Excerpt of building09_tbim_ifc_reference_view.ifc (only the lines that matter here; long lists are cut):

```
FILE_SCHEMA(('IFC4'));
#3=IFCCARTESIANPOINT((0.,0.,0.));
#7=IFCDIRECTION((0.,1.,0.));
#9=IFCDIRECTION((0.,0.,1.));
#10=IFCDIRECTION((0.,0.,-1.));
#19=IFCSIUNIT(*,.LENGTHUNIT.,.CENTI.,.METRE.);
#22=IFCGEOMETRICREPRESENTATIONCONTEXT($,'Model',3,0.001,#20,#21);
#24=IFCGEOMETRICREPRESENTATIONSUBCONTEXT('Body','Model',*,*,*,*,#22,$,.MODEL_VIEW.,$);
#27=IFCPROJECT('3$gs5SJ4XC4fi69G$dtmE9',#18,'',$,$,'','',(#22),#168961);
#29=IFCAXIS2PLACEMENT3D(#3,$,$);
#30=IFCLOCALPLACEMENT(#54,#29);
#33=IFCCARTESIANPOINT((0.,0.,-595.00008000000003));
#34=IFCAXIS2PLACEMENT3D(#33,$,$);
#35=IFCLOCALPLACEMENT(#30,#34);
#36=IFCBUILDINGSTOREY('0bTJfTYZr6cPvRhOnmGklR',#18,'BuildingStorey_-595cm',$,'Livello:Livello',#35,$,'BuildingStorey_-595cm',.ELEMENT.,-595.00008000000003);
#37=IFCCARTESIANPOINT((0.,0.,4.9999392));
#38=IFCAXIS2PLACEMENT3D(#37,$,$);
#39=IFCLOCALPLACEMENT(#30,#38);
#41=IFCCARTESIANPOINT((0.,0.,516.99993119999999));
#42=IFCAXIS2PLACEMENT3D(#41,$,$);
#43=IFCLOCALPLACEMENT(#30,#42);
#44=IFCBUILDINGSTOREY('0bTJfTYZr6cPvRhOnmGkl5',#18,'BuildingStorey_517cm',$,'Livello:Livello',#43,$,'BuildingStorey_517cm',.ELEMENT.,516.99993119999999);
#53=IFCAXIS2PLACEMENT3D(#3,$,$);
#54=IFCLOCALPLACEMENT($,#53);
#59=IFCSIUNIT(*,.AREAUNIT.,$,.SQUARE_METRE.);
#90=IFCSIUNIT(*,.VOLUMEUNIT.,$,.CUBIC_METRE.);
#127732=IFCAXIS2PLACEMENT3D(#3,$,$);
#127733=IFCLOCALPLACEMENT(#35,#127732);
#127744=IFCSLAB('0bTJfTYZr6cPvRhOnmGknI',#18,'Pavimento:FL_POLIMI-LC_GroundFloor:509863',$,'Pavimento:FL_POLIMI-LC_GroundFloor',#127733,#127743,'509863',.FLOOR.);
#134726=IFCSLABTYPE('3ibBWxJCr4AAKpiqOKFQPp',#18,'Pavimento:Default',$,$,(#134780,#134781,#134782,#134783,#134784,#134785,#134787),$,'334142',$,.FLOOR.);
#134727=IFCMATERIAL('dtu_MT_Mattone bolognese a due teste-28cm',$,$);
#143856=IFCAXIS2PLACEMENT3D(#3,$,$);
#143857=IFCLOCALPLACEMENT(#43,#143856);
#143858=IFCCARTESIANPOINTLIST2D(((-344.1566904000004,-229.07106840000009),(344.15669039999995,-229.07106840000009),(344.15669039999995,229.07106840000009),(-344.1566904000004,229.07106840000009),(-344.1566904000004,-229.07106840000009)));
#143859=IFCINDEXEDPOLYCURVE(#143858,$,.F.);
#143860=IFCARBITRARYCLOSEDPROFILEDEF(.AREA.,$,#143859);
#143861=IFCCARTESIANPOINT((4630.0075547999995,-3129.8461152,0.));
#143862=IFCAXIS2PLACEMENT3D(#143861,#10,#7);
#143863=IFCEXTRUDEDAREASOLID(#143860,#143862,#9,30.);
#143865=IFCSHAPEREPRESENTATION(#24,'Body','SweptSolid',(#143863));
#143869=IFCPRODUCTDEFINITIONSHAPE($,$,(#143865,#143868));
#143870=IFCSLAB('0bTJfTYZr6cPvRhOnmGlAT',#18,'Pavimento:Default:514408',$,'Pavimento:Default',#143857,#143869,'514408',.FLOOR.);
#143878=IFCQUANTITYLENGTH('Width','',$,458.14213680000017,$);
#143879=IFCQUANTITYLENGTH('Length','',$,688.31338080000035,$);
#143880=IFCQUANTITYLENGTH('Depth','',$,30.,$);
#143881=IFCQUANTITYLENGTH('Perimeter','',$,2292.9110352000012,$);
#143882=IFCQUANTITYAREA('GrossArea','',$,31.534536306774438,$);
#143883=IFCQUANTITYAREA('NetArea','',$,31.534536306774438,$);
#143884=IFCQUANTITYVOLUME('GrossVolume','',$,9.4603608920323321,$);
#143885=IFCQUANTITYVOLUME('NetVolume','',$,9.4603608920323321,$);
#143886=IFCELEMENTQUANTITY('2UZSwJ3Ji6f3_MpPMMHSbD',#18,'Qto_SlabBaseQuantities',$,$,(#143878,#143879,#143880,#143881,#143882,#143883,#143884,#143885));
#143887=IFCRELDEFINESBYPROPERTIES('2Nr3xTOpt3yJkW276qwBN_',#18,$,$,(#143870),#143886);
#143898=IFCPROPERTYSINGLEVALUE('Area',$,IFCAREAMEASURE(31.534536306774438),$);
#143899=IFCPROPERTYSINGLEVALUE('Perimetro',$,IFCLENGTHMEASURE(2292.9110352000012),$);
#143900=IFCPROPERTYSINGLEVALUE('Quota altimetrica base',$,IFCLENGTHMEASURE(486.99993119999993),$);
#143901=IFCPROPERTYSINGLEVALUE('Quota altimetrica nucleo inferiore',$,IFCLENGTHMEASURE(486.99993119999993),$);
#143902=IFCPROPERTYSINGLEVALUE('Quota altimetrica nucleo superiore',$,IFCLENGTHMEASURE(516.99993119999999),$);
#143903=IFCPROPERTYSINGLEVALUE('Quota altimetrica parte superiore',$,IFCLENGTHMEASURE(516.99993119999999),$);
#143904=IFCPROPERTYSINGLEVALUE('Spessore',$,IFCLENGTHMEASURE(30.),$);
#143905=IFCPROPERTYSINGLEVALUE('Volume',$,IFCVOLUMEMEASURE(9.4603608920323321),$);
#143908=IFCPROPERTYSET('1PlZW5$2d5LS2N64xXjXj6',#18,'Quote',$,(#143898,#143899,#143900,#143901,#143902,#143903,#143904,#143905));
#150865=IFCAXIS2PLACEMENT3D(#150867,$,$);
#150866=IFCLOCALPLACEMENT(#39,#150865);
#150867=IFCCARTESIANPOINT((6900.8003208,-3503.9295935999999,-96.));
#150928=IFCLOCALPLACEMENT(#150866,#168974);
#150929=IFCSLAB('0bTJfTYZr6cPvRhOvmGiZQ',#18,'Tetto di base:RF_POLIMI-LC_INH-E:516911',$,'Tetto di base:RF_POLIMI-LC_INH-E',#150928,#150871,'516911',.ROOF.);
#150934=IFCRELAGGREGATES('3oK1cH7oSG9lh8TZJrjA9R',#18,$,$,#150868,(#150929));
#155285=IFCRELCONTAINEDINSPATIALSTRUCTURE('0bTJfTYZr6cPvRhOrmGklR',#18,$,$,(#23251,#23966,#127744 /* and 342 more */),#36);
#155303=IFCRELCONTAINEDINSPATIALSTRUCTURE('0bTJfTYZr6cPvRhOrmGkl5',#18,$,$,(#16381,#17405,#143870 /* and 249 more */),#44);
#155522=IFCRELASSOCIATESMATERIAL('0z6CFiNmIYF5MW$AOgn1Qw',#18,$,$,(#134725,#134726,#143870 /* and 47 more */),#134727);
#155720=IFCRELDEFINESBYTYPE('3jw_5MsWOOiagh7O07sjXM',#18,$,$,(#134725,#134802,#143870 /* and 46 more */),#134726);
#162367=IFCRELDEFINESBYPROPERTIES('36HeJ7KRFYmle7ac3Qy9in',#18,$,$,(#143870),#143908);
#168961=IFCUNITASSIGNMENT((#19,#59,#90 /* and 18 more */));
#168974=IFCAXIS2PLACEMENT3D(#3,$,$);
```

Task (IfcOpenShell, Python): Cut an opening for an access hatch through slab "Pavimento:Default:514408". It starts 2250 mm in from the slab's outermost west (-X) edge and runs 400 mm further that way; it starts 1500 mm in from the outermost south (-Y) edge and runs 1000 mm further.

```python
import numpy as np
import ifcopenshell
import ifcopenshell.api.feature
import ifcopenshell.api.geometry
import ifcopenshell.api.pset
import ifcopenshell.api.root
import ifcopenshell.geom
import ifcopenshell.util.element
import ifcopenshell.util.placement
import ifcopenshell.util.representation
import ifcopenshell.util.shape
import ifcopenshell.util.unit

model = ifcopenshell.open("building09_tbim_ifc_reference_view.ifc")
unit_scale = ifcopenshell.util.unit.calculate_unit_scale(model)
area_scale = ifcopenshell.util.unit.calculate_unit_scale(model, "AREAUNIT")
volume_scale = ifcopenshell.util.unit.calculate_unit_scale(model, "VOLUMEUNIT")
settings = ifcopenshell.geom.settings()


def volume(element):
    """Net volume in cubic metres, openings subtracted."""
    shape = ifcopenshell.geom.create_shape(settings, element)
    return ifcopenshell.util.shape.get_volume(shape.geometry)


slab = model.by_guid("0bTJfTYZr6cPvRhOnmGlAT")
before = volume(slab)

# Extent in the slab's own axes, in metres. The edges named are its -X and -Y sides.
slab_shape = ifcopenshell.geom.create_shape(settings, slab)
vertices = ifcopenshell.util.shape.get_vertices(slab_shape.geometry)
x_min, y_min, bottom = vertices.min(axis=0)
top = vertices[:, 2].max()

opening = ifcopenshell.api.root.create_entity(model, ifc_class="IfcOpeningElement", name="Access hatch opening", predefined_type="OPENING")
context = ifcopenshell.util.representation.get_context(model, "Model", "Body", "MODEL_VIEW")
width, depth = 0.4, 1
outline = [(0.0, 0.0), (width, 0.0), (width, depth), (0.0, depth), (0.0, 0.0)]
# Overshoot both faces by 50 mm so the cut is clean.
shape = ifcopenshell.api.geometry.add_slab_representation(
    model, context=context, depth=top - bottom + 0.1, polyline=outline
)
ifcopenshell.api.geometry.assign_representation(model, product=opening, representation=shape)

matrix = ifcopenshell.util.placement.get_local_placement(slab.ObjectPlacement)
matrix[:, 3] = matrix @ np.append(np.array([x_min + 2.25, y_min + 1.5, bottom - 0.05]) / unit_scale, 1.0)
ifcopenshell.api.geometry.edit_object_placement(model, product=opening, matrix=matrix, is_si=False)
ifcopenshell.api.feature.add_feature(model, feature=opening, element=slab)

after = volume(slab)

# Update the slab's stored quantities.
qto = model.by_id(ifcopenshell.util.element.get_pset(slab, "Qto_SlabBaseQuantities", should_inherit=False)["id"])
ifcopenshell.api.pset.edit_qto(model, qto=qto, properties={
    "NetArea": after / (top - bottom) / area_scale,
    "NetVolume": after / volume_scale,
})
pset = model.by_id(ifcopenshell.util.element.get_pset(slab, "Quote", should_inherit=False)["id"])
ifcopenshell.api.pset.edit_pset(model, pset=pset, properties={
    "Area": model.create_entity("IfcAreaMeasure", after / (top - bottom) / area_scale),
    "Volume": model.create_entity("IfcVolumeMeasure", after / volume_scale),
})

print(f"slab volume {before:.3f} -> {after:.3f} m3")

model.write("building09_tbim_ifc_reference_view_updated.ifc")
```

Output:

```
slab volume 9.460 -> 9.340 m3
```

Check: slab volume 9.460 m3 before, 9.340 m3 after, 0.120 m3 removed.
